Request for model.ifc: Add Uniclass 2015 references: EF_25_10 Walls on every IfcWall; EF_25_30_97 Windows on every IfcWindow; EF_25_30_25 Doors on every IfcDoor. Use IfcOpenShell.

First a look at what the model holds.

```python
import ifcopenshell

model = ifcopenshell.open("model.ifc")
print(model.schema)
print("classifications:", [c.Name for c in model.by_type("IfcClassification")])
for ifc_class in ("IfcDoor", "IfcRoof", "IfcStair", "IfcWall", "IfcWindow"):
    print(ifc_class, len(model.by_type(ifc_class)))
```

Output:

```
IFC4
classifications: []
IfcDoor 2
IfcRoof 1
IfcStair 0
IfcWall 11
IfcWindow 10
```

```python
import ifcopenshell
import ifcopenshell.api.classification

model = ifcopenshell.open("model.ifc")

system = ifcopenshell.api.classification.add_classification(model, classification="Uniclass 2015")

codes = {
    "IfcWall": ("EF_25_10", "Walls"),
    "IfcWindow": ("EF_25_30_97", "Windows"),
    "IfcDoor": ("EF_25_30_25", "Doors"),
}
for ifc_class, (code, name) in codes.items():
    products = model.by_type(ifc_class)
    ifcopenshell.api.classification.add_reference(
        model, products=products, classification=system, identification=code, name=name
    )
    print(code, len(products))

model.write("model_edited.ifc")
```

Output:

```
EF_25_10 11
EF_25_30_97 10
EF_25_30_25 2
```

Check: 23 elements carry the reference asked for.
